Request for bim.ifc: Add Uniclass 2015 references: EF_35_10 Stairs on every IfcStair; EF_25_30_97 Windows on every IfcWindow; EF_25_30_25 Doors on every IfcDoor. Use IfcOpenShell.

First a look at what the model holds.

```python
import ifcopenshell

model = ifcopenshell.open("bim.ifc")
print(model.schema)
print("classifications:", [c.Name for c in model.by_type("IfcClassification")])
for ifc_class in ("IfcDoor", "IfcRoof", "IfcStair", "IfcWall", "IfcWindow"):
    print(ifc_class, len(model.by_type(ifc_class)))
```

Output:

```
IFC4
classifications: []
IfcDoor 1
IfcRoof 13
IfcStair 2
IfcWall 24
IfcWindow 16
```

```python
import ifcopenshell
import ifcopenshell.api.classification

model = ifcopenshell.open("bim.ifc")

system = ifcopenshell.api.classification.add_classification(model, classification="Uniclass 2015")

codes = {
    "IfcStair": ("EF_35_10", "Stairs"),
    "IfcWindow": ("EF_25_30_97", "Windows"),
    "IfcDoor": ("EF_25_30_25", "Doors"),
}
for ifc_class, (code, name) in codes.items():
    products = model.by_type(ifc_class)
    ifcopenshell.api.classification.add_reference(
        model, products=products, classification=system, identification=code, name=name
    )
    print(code, len(products))

model.write("bim_v2.ifc")
```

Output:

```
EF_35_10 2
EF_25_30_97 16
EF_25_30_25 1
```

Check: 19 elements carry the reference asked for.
